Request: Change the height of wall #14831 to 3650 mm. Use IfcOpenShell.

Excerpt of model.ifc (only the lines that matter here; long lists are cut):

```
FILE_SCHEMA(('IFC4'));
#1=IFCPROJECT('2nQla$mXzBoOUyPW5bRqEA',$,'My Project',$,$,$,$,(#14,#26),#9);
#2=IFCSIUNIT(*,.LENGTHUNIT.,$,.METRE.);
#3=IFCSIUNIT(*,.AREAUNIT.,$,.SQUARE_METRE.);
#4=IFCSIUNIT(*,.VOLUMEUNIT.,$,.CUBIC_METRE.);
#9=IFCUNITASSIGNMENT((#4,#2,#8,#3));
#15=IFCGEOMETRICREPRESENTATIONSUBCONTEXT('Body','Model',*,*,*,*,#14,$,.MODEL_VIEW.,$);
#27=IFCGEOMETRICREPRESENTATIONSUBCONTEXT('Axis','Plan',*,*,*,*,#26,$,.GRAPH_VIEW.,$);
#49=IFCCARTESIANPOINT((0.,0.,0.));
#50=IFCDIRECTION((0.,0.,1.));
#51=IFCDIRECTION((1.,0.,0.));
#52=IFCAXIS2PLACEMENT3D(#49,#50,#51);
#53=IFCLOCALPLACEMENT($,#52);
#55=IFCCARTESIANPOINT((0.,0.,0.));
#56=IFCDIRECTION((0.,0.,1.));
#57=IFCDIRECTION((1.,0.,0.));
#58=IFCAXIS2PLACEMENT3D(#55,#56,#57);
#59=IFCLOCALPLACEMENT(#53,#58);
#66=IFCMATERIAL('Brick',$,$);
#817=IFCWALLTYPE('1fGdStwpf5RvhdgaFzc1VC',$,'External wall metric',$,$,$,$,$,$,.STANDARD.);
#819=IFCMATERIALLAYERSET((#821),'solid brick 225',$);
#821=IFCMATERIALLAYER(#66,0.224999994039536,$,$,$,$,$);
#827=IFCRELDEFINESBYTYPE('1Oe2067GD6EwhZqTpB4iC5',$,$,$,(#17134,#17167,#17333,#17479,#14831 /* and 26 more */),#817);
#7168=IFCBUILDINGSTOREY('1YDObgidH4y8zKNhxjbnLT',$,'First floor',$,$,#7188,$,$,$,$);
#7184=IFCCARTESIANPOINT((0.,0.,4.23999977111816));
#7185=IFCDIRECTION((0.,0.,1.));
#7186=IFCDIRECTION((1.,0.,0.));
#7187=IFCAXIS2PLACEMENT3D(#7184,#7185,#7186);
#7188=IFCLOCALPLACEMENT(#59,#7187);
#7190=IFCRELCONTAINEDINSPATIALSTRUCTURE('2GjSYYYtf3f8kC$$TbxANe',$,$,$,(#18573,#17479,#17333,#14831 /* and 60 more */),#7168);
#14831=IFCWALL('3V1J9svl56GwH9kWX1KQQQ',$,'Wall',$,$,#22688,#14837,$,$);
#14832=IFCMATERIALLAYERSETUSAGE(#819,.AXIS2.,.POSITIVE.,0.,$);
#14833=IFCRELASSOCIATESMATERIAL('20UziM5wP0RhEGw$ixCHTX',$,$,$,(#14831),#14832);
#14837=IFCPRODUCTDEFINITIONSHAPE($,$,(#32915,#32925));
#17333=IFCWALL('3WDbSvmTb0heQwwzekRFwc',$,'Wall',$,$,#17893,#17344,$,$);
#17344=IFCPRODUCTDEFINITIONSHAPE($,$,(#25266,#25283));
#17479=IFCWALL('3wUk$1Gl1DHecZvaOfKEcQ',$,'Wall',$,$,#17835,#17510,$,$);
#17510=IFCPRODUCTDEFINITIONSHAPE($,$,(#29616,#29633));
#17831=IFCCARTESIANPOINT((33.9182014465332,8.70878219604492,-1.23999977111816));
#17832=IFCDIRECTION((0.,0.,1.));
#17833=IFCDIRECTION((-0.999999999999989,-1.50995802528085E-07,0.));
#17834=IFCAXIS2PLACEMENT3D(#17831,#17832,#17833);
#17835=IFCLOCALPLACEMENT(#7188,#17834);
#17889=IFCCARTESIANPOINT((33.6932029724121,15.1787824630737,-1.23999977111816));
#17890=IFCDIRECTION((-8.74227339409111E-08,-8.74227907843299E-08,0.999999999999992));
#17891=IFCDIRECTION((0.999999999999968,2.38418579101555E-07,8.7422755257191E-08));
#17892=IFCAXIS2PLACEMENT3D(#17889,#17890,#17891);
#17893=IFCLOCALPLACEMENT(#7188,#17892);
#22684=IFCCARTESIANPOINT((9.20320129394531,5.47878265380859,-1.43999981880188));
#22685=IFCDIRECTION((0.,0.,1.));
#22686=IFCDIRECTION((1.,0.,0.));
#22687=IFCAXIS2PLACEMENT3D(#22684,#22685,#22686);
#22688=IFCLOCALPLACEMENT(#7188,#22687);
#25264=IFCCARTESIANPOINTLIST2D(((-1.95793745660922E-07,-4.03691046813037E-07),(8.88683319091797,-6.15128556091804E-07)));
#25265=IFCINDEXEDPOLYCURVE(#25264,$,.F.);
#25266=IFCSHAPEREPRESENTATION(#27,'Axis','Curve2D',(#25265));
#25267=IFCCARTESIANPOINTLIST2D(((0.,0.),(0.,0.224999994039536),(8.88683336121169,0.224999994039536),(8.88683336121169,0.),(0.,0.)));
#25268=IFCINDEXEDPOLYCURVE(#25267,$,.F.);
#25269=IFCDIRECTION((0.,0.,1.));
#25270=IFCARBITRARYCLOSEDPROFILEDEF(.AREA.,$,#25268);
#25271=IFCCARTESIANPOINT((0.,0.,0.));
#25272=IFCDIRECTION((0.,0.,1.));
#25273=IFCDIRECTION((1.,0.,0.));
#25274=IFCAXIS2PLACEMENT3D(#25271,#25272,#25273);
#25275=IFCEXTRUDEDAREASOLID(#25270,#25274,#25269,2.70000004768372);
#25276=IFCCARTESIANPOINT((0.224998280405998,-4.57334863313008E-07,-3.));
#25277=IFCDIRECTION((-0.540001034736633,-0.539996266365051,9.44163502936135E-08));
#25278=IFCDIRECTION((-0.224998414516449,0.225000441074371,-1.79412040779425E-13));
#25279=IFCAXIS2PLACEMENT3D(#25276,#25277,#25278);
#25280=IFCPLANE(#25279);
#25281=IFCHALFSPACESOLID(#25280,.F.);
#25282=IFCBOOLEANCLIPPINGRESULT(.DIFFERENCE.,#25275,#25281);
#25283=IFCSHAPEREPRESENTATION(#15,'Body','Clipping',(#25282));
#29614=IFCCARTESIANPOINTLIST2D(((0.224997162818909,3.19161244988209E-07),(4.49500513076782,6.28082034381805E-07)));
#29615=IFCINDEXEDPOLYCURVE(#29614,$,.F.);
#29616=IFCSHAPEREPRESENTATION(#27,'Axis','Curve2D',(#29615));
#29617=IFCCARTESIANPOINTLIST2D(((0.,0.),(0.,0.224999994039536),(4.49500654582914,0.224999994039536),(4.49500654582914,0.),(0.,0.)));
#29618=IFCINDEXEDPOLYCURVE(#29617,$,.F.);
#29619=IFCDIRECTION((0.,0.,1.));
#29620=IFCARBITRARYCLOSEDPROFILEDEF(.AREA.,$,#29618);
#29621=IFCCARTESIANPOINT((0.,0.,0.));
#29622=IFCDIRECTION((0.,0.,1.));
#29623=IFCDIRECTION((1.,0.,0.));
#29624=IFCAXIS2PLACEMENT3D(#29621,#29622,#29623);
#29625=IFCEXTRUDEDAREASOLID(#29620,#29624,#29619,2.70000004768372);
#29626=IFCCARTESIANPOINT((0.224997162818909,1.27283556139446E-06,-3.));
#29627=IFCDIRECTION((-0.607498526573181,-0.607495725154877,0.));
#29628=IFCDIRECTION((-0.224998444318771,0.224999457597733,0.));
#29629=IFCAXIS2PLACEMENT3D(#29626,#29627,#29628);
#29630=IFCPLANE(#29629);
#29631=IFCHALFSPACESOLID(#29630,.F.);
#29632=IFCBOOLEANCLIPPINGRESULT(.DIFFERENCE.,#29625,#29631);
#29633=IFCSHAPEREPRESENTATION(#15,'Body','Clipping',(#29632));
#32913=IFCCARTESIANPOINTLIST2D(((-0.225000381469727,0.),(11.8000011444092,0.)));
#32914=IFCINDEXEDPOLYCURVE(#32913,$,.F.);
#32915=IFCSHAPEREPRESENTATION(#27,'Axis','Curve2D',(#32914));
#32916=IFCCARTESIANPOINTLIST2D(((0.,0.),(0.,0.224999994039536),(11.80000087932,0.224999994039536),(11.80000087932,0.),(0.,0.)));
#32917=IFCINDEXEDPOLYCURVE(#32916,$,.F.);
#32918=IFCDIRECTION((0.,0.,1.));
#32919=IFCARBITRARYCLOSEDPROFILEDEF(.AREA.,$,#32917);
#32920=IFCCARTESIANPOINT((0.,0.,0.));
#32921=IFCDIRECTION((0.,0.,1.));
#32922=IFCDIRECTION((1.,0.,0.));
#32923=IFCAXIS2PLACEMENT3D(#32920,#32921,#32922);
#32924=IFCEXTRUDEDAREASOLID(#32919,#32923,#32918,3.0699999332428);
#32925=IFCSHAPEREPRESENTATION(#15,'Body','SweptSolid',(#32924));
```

```python
import ifcopenshell
import ifcopenshell.geom
import ifcopenshell.util.representation
import ifcopenshell.util.shape
import ifcopenshell.util.unit

model = ifcopenshell.open("model.ifc")
unit_scale = ifcopenshell.util.unit.calculate_unit_scale(model)
settings = ifcopenshell.geom.settings()


def volume(element):
    """Net volume in cubic metres, openings subtracted."""
    shape = ifcopenshell.geom.create_shape(settings, element)
    return ifcopenshell.util.shape.get_volume(shape.geometry)


wall = model.by_guid("3V1J9svl56GwH9kWX1KQQQ")
before = volume(wall)

body = ifcopenshell.util.representation.get_representation(wall, "Model", "Body")
solid = body.Items[0]
old_height = solid.Depth
solid.Depth = 3.65 / unit_scale
after = volume(wall)

print(f"height {old_height:g} -> {solid.Depth:g}, volume {before:.3f} -> {after:.3f} m3")

model.write("model-out.ifc")
```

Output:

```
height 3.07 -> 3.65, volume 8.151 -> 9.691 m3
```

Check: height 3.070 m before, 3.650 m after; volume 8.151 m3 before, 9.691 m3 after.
